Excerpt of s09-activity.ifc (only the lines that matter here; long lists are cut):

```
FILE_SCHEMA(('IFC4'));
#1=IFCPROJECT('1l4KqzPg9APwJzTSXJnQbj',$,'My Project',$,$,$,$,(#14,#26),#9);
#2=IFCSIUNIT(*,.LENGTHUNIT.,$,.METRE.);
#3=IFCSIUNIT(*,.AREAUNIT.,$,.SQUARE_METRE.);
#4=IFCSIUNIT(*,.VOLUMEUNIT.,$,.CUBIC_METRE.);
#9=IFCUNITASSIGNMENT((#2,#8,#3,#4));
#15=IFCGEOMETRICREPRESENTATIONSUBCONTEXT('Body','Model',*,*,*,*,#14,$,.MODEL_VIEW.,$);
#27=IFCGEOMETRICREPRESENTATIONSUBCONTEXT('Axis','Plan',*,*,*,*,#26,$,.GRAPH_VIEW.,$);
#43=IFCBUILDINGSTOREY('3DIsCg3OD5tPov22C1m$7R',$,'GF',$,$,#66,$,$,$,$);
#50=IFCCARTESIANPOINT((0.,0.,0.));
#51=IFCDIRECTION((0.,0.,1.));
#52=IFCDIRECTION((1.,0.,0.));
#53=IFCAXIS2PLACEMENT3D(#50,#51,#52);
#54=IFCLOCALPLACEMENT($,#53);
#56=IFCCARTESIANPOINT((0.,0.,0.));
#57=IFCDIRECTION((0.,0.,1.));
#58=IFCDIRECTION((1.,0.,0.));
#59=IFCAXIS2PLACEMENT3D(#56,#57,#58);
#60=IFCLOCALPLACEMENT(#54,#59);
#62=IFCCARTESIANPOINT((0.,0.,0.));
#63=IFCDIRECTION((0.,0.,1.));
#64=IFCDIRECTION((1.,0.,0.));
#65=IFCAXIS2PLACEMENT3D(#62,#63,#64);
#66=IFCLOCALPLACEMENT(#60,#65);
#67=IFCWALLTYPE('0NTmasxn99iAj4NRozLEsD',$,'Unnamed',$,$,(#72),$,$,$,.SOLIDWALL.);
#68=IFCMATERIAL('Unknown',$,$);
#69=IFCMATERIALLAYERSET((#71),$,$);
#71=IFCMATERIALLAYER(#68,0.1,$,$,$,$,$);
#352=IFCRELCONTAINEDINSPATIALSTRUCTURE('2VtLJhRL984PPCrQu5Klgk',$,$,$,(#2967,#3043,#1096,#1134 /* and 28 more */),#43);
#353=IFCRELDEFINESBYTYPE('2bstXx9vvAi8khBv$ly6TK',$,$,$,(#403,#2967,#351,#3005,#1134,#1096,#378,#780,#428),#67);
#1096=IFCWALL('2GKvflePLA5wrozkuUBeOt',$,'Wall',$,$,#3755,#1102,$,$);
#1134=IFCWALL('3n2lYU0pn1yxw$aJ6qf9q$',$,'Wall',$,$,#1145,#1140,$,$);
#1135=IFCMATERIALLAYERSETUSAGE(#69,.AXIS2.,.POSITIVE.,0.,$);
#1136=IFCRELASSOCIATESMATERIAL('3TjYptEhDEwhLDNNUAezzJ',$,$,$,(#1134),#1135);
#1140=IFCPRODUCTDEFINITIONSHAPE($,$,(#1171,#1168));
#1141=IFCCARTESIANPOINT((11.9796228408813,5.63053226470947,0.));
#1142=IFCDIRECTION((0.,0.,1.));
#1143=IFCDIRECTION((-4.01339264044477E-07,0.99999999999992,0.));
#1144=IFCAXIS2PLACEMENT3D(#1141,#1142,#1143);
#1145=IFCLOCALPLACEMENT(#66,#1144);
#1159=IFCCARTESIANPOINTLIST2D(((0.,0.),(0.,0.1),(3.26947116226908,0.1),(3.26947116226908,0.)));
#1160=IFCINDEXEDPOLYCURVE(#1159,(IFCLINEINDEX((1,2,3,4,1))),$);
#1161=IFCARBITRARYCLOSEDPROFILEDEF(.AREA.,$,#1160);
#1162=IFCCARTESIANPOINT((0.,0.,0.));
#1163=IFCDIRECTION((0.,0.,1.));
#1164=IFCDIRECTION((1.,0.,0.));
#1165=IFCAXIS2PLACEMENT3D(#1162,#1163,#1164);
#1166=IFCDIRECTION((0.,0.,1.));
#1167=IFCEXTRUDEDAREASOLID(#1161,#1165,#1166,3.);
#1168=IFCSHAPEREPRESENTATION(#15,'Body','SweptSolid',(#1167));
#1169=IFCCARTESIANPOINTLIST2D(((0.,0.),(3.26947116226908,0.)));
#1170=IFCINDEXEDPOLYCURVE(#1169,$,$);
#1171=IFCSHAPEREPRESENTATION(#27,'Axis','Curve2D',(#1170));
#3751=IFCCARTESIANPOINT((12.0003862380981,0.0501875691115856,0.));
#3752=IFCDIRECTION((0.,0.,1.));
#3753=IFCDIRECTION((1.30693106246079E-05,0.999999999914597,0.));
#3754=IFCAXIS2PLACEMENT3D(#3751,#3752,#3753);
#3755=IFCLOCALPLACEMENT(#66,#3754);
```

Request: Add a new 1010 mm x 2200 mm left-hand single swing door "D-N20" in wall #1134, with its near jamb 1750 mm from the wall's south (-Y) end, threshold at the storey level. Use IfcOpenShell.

```python
import numpy as np
import ifcopenshell
import ifcopenshell.api.feature
import ifcopenshell.api.geometry
import ifcopenshell.api.root
import ifcopenshell.api.spatial
import ifcopenshell.geom
import ifcopenshell.util.element
import ifcopenshell.util.placement
import ifcopenshell.util.representation
import ifcopenshell.util.shape
import ifcopenshell.util.unit

model = ifcopenshell.open("s09-activity.ifc")
unit_scale = ifcopenshell.util.unit.calculate_unit_scale(model)
settings = ifcopenshell.geom.settings()


def volume(element):
    """Net volume in cubic metres, openings subtracted."""
    shape = ifcopenshell.geom.create_shape(settings, element)
    return ifcopenshell.util.shape.get_volume(shape.geometry)


wall = model.by_guid("3n2lYU0pn1yxw$aJ6qf9q$")
storey = ifcopenshell.util.element.get_container(wall, ifc_class="IfcBuildingStorey")
context = ifcopenshell.util.representation.get_context(model, "Model", "Body", "MODEL_VIEW")
before = volume(wall)

width, height, from_end, sill = 1.01, 2.2, 1.75, 0.0  # metres

# The wall runs along its own X axis, and the end named is its -X end.
wall_shape = ifcopenshell.geom.create_shape(settings, wall)
x, y, z = ifcopenshell.util.shape.get_vertices(wall_shape.geometry).T
start = x.min() + from_end
face, thickness = float(y.min()), float(y.max() - y.min())
wall_matrix = ifcopenshell.util.placement.get_local_placement(wall.ObjectPlacement)
level = ifcopenshell.util.placement.get_local_placement(storey.ObjectPlacement)[2, 3]


def in_wall(x, y):
    """Placement at x, y metres in the wall's axes, at sill height."""
    matrix = wall_matrix.copy()
    matrix[:, 3] = wall_matrix @ np.array([x / unit_scale, y / unit_scale, 0.0, 1.0])
    matrix[2, 3] = level + sill / unit_scale
    return matrix


# Opening: a box that overshoots both wall faces by 50 mm.
opening = ifcopenshell.api.root.create_entity(model, ifc_class="IfcOpeningElement", predefined_type="OPENING")
box = ifcopenshell.api.geometry.add_wall_representation(
    model, context=context, length=width, height=height, thickness=thickness + 0.1
)
ifcopenshell.api.geometry.assign_representation(model, product=opening, representation=box)
ifcopenshell.api.geometry.edit_object_placement(model, product=opening, matrix=in_wall(start, face - 0.05), is_si=False)
ifcopenshell.api.feature.add_feature(model, feature=opening, element=wall)

door = ifcopenshell.api.root.create_entity(model, ifc_class="IfcDoor", name="D-N20", predefined_type="DOOR")
door.OverallWidth, door.OverallHeight = width / unit_scale, height / unit_scale
door.OperationType = "SINGLE_SWING_LEFT"
body = ifcopenshell.api.geometry.add_door_representation(
    model,
    context=context,
    overall_width=door.OverallWidth,
    overall_height=door.OverallHeight,
    operation_type="SINGLE_SWING_LEFT",
    lining_properties={"LiningDepth": thickness / unit_scale, "ThresholdDepth": thickness / unit_scale},
)
ifcopenshell.api.geometry.assign_representation(model, product=door, representation=body)
ifcopenshell.api.spatial.assign_container(model, products=[door], relating_structure=storey)
ifcopenshell.api.feature.add_filling(model, opening=opening, element=door)

# The lining spans the wall, so the door starts at the wall face.
ifcopenshell.api.geometry.edit_object_placement(model, product=door, matrix=in_wall(start, face), is_si=False)

after = volume(wall)

print(f"wall volume {before:.3f} -> {after:.3f} m3")

model.write("s09-activity_updated.ifc")
```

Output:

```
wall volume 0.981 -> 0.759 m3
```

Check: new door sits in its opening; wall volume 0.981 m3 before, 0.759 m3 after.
